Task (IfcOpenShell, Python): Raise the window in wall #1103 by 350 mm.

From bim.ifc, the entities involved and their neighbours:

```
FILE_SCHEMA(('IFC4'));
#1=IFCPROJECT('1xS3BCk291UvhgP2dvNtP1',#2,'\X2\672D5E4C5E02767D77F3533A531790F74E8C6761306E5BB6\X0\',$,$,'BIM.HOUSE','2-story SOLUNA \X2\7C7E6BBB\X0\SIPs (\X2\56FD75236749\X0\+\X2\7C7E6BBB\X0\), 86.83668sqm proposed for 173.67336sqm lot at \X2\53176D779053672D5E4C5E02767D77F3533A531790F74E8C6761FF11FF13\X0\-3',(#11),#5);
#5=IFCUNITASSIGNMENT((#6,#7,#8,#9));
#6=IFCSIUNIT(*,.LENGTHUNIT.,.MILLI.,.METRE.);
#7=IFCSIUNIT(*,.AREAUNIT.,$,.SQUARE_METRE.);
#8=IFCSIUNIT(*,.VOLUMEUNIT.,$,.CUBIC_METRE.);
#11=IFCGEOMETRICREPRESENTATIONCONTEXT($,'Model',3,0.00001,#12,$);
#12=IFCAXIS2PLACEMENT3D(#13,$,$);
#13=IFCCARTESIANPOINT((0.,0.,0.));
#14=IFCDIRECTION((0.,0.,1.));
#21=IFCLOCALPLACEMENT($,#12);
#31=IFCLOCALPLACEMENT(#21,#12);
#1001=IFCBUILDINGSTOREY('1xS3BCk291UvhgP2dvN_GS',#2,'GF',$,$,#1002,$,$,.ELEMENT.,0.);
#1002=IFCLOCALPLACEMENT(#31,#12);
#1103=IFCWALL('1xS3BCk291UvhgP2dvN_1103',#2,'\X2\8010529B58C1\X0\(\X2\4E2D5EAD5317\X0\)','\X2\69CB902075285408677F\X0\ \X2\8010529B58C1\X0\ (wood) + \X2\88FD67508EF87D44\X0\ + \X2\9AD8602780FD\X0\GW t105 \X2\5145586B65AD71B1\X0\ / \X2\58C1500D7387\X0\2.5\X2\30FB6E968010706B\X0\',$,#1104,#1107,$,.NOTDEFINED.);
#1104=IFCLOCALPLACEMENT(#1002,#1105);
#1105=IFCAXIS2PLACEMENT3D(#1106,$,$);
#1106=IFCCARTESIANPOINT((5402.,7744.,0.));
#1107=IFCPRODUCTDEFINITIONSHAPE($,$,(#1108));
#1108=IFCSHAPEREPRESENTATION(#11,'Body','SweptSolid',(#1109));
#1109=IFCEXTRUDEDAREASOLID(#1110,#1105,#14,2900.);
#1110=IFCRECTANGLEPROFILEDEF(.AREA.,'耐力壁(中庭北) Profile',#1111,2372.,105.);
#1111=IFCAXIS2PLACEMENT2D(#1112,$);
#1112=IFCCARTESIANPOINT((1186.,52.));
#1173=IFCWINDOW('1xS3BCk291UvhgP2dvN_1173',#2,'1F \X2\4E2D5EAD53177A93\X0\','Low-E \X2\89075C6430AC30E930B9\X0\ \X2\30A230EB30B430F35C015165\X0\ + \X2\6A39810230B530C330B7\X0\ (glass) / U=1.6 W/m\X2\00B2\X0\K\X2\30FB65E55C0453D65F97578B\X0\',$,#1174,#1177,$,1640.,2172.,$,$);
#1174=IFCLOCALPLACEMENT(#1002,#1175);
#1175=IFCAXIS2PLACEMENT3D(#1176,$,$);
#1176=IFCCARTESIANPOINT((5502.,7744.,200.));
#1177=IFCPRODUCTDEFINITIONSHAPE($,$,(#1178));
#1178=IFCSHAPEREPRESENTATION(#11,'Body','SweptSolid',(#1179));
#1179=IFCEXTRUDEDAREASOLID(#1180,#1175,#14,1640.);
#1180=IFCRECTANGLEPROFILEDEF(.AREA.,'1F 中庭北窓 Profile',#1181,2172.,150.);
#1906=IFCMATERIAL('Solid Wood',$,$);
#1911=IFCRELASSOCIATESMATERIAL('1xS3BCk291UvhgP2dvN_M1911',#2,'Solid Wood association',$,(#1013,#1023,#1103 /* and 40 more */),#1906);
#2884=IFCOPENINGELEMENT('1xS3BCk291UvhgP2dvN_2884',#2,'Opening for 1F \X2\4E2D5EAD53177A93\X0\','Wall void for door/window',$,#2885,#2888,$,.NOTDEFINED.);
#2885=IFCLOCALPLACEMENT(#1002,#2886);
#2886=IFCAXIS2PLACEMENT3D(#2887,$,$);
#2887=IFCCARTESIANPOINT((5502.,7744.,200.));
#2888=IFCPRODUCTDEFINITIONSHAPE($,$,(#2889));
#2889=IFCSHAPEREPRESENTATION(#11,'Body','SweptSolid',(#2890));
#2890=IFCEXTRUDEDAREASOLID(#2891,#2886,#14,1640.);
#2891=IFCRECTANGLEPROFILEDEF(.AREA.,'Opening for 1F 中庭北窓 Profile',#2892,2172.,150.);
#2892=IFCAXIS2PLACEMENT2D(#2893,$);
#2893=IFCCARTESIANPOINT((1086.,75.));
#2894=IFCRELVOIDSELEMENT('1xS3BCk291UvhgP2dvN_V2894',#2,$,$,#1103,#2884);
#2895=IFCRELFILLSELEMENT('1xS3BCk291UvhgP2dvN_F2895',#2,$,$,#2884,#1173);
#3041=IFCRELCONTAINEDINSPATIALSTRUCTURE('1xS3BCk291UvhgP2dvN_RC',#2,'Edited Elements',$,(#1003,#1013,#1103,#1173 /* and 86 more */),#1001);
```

```python
import numpy as np
import ifcopenshell
import ifcopenshell.api.geometry
import ifcopenshell.util.placement
import ifcopenshell.util.unit

model = ifcopenshell.open("bim.ifc")
unit_scale = ifcopenshell.util.unit.calculate_unit_scale(model)

window = model.by_id(1173)
opening = window.FillsVoids[0].RelatingOpeningElement
dz = 0.35 / unit_scale

shift = np.array([0.0, 0.0, dz])
# The window is not placed relative to its opening, so move both.
for product in (opening, window):
    matrix = ifcopenshell.util.placement.get_local_placement(product.ObjectPlacement)
    matrix[:3, 3] += shift
    ifcopenshell.api.geometry.edit_object_placement(model, product=product, matrix=matrix, is_si=False)

print(f"moved by {dz * unit_scale:+.3f} m")

model.write("bim_updated.ifc")
```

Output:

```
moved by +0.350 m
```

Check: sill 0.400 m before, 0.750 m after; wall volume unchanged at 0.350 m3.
